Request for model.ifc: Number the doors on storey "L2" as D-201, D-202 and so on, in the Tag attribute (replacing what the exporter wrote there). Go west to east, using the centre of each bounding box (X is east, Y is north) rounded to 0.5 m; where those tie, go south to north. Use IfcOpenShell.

First a look at what the model holds.

```python
import ifcopenshell
import ifcopenshell.util.element
import ifcopenshell.util.placement

model = ifcopenshell.open("model.ifc")
print(model.schema)
storey = next(s for s in model.by_type("IfcBuildingStorey") if s.Name == "L2")
doors = [e for e in ifcopenshell.util.element.get_decomposition(storey) if e.is_a("IfcDoor")]
for e in sorted(doors, key=lambda e: e.id()):
    origin = ifcopenshell.util.placement.get_local_placement(e.ObjectPlacement)[:3, 3]
    print(e.id(), e.Tag, e.Name, origin.round(2) + 0.0, sep=" | ")
```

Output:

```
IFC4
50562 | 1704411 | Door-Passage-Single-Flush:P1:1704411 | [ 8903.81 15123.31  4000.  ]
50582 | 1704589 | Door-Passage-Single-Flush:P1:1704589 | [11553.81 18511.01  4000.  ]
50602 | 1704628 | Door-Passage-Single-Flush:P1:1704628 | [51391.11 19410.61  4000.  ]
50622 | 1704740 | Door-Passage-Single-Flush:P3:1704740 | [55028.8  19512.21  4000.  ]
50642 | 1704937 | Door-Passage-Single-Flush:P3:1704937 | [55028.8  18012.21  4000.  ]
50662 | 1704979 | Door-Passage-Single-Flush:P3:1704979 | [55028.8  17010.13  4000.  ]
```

```python
import ifcopenshell
import ifcopenshell.geom
import ifcopenshell.util.element
import ifcopenshell.util.shape

model = ifcopenshell.open("model.ifc")
settings = ifcopenshell.geom.settings()
settings.set("use-world-coords", True)


def centre(element):
    shape = ifcopenshell.geom.create_shape(settings, element)
    return ifcopenshell.util.shape.get_bbox_centroid(shape.geometry)


storey = next(s for s in model.by_type("IfcBuildingStorey") if s.Name == "L2")
doors = [e for e in ifcopenshell.util.element.get_decomposition(storey) if e.is_a("IfcDoor")]

# Insertion points can sit at a corner or the storey origin, so sort by the geometry (in metres).
centres = {e: centre(e) for e in doors}
doors.sort(key=lambda e: (round(centres[e][0] / 0.5), centres[e][1]))

for i, e in enumerate(doors, start=1):
    number = f"D-2{i:02d}"
    e.Tag = number
    print(e.id(), number)

model.write("model_updated.ifc")
```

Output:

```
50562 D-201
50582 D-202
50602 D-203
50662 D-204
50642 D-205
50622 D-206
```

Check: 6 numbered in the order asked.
